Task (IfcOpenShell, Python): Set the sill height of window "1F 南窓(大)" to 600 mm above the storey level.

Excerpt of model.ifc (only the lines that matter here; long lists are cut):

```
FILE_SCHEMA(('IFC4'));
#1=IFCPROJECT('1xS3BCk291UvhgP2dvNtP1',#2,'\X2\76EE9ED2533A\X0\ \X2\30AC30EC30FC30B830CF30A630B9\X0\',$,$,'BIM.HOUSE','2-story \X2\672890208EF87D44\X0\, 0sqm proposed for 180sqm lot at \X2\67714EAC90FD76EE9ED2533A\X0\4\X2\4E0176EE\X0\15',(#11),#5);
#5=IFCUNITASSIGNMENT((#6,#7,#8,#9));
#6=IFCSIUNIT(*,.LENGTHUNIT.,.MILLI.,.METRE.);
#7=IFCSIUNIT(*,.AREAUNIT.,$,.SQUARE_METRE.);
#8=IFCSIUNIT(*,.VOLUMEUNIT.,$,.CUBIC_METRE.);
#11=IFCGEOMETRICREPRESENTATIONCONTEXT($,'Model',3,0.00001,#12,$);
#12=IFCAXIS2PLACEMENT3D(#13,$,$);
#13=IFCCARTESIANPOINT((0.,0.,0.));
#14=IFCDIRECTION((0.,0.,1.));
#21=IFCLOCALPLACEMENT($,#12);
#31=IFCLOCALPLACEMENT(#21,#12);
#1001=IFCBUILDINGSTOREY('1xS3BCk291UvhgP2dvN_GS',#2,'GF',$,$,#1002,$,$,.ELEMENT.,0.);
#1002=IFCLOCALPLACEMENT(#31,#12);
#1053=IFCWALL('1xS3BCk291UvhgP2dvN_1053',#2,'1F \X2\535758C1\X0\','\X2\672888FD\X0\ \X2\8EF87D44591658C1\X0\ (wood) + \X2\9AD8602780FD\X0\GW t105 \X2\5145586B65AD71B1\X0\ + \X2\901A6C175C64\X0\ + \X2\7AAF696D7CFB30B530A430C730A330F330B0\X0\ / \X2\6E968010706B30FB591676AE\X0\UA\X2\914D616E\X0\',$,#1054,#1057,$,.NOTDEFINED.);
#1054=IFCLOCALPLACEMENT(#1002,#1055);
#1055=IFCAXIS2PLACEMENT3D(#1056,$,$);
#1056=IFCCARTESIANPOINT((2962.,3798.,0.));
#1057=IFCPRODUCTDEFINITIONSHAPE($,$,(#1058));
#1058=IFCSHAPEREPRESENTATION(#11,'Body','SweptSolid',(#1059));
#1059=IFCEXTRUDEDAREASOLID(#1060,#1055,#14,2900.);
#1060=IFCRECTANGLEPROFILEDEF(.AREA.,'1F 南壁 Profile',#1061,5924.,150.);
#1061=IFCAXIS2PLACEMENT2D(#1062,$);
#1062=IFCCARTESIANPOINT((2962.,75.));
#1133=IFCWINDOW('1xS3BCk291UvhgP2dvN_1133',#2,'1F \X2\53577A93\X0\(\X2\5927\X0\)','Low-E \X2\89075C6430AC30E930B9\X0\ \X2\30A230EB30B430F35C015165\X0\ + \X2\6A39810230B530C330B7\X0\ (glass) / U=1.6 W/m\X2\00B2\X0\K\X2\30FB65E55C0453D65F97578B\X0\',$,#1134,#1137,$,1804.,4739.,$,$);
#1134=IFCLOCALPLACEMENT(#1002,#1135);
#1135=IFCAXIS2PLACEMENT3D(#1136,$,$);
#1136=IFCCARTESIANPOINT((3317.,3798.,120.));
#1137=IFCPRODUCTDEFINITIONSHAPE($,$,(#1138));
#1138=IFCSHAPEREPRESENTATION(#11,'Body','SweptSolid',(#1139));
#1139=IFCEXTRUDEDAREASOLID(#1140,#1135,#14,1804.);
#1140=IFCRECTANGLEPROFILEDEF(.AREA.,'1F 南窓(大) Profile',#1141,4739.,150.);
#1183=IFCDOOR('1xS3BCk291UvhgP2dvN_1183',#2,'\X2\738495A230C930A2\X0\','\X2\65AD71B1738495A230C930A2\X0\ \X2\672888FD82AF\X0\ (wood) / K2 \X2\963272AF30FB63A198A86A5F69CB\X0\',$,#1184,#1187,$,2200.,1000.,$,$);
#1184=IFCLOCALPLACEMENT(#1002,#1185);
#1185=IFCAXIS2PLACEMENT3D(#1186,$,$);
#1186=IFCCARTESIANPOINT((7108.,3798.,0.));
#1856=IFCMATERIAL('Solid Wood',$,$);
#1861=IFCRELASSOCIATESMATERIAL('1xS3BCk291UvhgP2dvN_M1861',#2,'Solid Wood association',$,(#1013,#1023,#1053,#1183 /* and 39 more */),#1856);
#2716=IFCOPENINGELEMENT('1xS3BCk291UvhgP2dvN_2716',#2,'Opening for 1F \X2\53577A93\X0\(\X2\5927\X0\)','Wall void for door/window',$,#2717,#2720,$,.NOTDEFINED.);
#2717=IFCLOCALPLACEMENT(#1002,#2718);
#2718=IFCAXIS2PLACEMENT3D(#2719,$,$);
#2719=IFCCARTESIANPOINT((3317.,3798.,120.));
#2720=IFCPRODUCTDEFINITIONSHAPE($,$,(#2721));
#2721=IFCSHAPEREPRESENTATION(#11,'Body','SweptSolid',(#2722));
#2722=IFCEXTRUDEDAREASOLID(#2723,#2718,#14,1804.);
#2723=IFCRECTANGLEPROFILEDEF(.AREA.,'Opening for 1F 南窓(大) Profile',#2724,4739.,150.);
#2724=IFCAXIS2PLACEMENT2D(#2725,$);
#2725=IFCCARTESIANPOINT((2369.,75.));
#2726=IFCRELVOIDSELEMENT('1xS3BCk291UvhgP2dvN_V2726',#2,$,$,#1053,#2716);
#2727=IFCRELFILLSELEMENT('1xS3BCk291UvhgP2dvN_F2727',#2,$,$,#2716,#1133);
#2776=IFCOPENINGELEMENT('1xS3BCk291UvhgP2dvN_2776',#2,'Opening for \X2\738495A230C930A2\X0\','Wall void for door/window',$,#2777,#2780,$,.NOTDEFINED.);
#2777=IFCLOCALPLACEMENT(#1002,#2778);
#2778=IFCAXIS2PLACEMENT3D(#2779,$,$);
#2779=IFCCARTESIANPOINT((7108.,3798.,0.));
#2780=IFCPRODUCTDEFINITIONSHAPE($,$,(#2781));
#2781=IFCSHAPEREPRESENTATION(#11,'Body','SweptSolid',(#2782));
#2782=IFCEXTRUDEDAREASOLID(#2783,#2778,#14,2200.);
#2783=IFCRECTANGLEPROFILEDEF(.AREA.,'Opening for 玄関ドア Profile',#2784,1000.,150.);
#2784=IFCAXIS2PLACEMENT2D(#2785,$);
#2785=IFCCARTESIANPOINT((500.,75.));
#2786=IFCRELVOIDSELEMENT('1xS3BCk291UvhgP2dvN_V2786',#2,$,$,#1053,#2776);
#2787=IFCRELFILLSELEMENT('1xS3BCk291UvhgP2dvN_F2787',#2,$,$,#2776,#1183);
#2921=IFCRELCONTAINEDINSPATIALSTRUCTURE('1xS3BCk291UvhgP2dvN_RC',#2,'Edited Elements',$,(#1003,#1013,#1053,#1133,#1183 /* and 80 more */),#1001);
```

```python
import numpy as np
import ifcopenshell
import ifcopenshell.api.geometry
import ifcopenshell.geom
import ifcopenshell.util.element
import ifcopenshell.util.placement
import ifcopenshell.util.shape
import ifcopenshell.util.unit

model = ifcopenshell.open("model.ifc")
unit_scale = ifcopenshell.util.unit.calculate_unit_scale(model)

window = model.by_guid("1xS3BCk291UvhgP2dvN_1133")
opening = window.FillsVoids[0].RelatingOpeningElement
storey = ifcopenshell.util.element.get_container(window, ifc_class="IfcBuildingStorey")
level = ifcopenshell.util.placement.get_local_placement(storey.ObjectPlacement)[2, 3]

# The opening's origin need not be at the sill, so measure its lowest point.
shape = ifcopenshell.geom.create_shape(ifcopenshell.geom.settings(), opening)
bottom = ifcopenshell.util.shape.get_shape_bottom_elevation(shape, shape.geometry) / unit_scale
dz = level + 0.6 / unit_scale - bottom

shift = np.array([0.0, 0.0, dz])
# The window is not placed relative to its opening, so move both.
for product in (opening, window):
    matrix = ifcopenshell.util.placement.get_local_placement(product.ObjectPlacement)
    matrix[:3, 3] += shift
    ifcopenshell.api.geometry.edit_object_placement(model, product=product, matrix=matrix, is_si=False)

print(f"moved by {dz * unit_scale:+.3f} m")

model.write("model_rev.ifc")
```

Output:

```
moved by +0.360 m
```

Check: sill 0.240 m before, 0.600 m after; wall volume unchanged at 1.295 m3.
